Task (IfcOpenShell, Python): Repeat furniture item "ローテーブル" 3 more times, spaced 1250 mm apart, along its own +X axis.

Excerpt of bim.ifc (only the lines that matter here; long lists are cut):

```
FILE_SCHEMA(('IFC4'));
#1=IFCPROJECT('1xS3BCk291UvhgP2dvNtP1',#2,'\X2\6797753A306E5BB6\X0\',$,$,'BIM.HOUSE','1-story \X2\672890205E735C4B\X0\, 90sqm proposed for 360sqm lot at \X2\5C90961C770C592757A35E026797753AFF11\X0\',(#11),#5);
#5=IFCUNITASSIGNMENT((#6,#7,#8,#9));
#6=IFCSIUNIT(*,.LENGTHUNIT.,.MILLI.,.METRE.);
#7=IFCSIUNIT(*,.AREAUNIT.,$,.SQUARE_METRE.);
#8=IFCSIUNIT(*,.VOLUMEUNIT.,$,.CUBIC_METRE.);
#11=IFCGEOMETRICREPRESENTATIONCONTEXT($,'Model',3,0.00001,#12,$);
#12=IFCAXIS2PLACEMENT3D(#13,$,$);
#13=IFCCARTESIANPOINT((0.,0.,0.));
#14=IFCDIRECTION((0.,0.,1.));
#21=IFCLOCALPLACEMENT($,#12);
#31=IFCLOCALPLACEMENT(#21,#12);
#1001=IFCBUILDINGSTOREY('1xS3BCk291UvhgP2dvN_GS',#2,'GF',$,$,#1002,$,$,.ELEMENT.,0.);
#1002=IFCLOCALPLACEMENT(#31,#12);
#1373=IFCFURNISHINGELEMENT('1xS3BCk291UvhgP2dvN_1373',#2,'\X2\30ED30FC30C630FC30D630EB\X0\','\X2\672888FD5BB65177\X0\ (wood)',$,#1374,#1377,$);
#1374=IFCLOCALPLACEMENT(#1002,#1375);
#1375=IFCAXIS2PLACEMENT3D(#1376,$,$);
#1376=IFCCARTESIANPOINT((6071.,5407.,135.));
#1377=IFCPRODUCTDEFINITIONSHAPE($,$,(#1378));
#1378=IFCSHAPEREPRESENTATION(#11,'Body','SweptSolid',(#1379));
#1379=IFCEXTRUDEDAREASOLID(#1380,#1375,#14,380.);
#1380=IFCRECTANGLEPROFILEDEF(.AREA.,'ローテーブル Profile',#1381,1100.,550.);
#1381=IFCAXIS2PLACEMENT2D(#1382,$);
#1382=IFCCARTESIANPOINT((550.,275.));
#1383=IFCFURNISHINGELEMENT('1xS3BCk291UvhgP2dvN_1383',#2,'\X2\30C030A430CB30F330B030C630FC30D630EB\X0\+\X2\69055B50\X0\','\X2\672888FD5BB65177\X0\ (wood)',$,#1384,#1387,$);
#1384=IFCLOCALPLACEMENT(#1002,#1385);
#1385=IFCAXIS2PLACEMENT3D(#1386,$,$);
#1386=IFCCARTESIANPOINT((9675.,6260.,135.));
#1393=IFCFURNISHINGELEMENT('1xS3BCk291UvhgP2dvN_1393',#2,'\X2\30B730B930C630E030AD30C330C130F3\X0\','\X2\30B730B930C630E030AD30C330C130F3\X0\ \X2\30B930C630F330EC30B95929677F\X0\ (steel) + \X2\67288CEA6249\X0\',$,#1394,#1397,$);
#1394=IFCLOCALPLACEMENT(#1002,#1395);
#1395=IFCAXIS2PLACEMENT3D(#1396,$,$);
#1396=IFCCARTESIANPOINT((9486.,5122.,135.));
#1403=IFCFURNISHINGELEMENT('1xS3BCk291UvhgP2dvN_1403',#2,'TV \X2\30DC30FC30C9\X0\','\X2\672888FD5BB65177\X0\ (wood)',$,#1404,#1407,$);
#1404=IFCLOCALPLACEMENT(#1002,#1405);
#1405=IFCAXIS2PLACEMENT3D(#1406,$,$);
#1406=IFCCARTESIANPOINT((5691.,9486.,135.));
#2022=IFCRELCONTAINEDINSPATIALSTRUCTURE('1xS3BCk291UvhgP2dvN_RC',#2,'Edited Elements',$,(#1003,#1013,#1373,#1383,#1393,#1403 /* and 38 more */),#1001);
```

```python
import ifcopenshell
import ifcopenshell.api.geometry
import ifcopenshell.api.root
import ifcopenshell.util.element
import ifcopenshell.util.placement
import ifcopenshell.util.unit

model = ifcopenshell.open("bim.ifc")
unit_scale = ifcopenshell.util.unit.calculate_unit_scale(model)


def reuse_history(source, copy):
    """copy_class also copies each property set's owner history, people and application; keep the originals."""
    for rel in copy.IsDefinedBy:
        if rel.is_a("IfcRelDefinesByProperties") and (history := rel.RelatingPropertyDefinition.OwnerHistory):
            rel.RelatingPropertyDefinition.OwnerHistory = source.OwnerHistory
            ifcopenshell.util.element.remove_deep2(model, history)


source = model.by_guid("1xS3BCk291UvhgP2dvN_1373")
base = ifcopenshell.util.placement.get_local_placement(source.ObjectPlacement)
step = base[:3, 0] * 1.25 / unit_scale

for i in range(1, 4):
    copy = ifcopenshell.api.root.copy_class(model, product=source)
    copy.Representation = ifcopenshell.util.element.copy_deep(
        model, source.Representation, exclude=["IfcGeometricRepresentationContext", "IfcRepresentationMap"]
    )
    reuse_history(source, copy)
    matrix = base.copy()
    matrix[:3, 3] += i * step
    print("added at", matrix[:3, 3].round(3) + 0.0)
    ifcopenshell.api.geometry.edit_object_placement(model, product=copy, matrix=matrix, is_si=False)

model.write("bim_v2.ifc")
```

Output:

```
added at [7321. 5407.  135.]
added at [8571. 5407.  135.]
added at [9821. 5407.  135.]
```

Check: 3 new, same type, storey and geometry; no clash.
